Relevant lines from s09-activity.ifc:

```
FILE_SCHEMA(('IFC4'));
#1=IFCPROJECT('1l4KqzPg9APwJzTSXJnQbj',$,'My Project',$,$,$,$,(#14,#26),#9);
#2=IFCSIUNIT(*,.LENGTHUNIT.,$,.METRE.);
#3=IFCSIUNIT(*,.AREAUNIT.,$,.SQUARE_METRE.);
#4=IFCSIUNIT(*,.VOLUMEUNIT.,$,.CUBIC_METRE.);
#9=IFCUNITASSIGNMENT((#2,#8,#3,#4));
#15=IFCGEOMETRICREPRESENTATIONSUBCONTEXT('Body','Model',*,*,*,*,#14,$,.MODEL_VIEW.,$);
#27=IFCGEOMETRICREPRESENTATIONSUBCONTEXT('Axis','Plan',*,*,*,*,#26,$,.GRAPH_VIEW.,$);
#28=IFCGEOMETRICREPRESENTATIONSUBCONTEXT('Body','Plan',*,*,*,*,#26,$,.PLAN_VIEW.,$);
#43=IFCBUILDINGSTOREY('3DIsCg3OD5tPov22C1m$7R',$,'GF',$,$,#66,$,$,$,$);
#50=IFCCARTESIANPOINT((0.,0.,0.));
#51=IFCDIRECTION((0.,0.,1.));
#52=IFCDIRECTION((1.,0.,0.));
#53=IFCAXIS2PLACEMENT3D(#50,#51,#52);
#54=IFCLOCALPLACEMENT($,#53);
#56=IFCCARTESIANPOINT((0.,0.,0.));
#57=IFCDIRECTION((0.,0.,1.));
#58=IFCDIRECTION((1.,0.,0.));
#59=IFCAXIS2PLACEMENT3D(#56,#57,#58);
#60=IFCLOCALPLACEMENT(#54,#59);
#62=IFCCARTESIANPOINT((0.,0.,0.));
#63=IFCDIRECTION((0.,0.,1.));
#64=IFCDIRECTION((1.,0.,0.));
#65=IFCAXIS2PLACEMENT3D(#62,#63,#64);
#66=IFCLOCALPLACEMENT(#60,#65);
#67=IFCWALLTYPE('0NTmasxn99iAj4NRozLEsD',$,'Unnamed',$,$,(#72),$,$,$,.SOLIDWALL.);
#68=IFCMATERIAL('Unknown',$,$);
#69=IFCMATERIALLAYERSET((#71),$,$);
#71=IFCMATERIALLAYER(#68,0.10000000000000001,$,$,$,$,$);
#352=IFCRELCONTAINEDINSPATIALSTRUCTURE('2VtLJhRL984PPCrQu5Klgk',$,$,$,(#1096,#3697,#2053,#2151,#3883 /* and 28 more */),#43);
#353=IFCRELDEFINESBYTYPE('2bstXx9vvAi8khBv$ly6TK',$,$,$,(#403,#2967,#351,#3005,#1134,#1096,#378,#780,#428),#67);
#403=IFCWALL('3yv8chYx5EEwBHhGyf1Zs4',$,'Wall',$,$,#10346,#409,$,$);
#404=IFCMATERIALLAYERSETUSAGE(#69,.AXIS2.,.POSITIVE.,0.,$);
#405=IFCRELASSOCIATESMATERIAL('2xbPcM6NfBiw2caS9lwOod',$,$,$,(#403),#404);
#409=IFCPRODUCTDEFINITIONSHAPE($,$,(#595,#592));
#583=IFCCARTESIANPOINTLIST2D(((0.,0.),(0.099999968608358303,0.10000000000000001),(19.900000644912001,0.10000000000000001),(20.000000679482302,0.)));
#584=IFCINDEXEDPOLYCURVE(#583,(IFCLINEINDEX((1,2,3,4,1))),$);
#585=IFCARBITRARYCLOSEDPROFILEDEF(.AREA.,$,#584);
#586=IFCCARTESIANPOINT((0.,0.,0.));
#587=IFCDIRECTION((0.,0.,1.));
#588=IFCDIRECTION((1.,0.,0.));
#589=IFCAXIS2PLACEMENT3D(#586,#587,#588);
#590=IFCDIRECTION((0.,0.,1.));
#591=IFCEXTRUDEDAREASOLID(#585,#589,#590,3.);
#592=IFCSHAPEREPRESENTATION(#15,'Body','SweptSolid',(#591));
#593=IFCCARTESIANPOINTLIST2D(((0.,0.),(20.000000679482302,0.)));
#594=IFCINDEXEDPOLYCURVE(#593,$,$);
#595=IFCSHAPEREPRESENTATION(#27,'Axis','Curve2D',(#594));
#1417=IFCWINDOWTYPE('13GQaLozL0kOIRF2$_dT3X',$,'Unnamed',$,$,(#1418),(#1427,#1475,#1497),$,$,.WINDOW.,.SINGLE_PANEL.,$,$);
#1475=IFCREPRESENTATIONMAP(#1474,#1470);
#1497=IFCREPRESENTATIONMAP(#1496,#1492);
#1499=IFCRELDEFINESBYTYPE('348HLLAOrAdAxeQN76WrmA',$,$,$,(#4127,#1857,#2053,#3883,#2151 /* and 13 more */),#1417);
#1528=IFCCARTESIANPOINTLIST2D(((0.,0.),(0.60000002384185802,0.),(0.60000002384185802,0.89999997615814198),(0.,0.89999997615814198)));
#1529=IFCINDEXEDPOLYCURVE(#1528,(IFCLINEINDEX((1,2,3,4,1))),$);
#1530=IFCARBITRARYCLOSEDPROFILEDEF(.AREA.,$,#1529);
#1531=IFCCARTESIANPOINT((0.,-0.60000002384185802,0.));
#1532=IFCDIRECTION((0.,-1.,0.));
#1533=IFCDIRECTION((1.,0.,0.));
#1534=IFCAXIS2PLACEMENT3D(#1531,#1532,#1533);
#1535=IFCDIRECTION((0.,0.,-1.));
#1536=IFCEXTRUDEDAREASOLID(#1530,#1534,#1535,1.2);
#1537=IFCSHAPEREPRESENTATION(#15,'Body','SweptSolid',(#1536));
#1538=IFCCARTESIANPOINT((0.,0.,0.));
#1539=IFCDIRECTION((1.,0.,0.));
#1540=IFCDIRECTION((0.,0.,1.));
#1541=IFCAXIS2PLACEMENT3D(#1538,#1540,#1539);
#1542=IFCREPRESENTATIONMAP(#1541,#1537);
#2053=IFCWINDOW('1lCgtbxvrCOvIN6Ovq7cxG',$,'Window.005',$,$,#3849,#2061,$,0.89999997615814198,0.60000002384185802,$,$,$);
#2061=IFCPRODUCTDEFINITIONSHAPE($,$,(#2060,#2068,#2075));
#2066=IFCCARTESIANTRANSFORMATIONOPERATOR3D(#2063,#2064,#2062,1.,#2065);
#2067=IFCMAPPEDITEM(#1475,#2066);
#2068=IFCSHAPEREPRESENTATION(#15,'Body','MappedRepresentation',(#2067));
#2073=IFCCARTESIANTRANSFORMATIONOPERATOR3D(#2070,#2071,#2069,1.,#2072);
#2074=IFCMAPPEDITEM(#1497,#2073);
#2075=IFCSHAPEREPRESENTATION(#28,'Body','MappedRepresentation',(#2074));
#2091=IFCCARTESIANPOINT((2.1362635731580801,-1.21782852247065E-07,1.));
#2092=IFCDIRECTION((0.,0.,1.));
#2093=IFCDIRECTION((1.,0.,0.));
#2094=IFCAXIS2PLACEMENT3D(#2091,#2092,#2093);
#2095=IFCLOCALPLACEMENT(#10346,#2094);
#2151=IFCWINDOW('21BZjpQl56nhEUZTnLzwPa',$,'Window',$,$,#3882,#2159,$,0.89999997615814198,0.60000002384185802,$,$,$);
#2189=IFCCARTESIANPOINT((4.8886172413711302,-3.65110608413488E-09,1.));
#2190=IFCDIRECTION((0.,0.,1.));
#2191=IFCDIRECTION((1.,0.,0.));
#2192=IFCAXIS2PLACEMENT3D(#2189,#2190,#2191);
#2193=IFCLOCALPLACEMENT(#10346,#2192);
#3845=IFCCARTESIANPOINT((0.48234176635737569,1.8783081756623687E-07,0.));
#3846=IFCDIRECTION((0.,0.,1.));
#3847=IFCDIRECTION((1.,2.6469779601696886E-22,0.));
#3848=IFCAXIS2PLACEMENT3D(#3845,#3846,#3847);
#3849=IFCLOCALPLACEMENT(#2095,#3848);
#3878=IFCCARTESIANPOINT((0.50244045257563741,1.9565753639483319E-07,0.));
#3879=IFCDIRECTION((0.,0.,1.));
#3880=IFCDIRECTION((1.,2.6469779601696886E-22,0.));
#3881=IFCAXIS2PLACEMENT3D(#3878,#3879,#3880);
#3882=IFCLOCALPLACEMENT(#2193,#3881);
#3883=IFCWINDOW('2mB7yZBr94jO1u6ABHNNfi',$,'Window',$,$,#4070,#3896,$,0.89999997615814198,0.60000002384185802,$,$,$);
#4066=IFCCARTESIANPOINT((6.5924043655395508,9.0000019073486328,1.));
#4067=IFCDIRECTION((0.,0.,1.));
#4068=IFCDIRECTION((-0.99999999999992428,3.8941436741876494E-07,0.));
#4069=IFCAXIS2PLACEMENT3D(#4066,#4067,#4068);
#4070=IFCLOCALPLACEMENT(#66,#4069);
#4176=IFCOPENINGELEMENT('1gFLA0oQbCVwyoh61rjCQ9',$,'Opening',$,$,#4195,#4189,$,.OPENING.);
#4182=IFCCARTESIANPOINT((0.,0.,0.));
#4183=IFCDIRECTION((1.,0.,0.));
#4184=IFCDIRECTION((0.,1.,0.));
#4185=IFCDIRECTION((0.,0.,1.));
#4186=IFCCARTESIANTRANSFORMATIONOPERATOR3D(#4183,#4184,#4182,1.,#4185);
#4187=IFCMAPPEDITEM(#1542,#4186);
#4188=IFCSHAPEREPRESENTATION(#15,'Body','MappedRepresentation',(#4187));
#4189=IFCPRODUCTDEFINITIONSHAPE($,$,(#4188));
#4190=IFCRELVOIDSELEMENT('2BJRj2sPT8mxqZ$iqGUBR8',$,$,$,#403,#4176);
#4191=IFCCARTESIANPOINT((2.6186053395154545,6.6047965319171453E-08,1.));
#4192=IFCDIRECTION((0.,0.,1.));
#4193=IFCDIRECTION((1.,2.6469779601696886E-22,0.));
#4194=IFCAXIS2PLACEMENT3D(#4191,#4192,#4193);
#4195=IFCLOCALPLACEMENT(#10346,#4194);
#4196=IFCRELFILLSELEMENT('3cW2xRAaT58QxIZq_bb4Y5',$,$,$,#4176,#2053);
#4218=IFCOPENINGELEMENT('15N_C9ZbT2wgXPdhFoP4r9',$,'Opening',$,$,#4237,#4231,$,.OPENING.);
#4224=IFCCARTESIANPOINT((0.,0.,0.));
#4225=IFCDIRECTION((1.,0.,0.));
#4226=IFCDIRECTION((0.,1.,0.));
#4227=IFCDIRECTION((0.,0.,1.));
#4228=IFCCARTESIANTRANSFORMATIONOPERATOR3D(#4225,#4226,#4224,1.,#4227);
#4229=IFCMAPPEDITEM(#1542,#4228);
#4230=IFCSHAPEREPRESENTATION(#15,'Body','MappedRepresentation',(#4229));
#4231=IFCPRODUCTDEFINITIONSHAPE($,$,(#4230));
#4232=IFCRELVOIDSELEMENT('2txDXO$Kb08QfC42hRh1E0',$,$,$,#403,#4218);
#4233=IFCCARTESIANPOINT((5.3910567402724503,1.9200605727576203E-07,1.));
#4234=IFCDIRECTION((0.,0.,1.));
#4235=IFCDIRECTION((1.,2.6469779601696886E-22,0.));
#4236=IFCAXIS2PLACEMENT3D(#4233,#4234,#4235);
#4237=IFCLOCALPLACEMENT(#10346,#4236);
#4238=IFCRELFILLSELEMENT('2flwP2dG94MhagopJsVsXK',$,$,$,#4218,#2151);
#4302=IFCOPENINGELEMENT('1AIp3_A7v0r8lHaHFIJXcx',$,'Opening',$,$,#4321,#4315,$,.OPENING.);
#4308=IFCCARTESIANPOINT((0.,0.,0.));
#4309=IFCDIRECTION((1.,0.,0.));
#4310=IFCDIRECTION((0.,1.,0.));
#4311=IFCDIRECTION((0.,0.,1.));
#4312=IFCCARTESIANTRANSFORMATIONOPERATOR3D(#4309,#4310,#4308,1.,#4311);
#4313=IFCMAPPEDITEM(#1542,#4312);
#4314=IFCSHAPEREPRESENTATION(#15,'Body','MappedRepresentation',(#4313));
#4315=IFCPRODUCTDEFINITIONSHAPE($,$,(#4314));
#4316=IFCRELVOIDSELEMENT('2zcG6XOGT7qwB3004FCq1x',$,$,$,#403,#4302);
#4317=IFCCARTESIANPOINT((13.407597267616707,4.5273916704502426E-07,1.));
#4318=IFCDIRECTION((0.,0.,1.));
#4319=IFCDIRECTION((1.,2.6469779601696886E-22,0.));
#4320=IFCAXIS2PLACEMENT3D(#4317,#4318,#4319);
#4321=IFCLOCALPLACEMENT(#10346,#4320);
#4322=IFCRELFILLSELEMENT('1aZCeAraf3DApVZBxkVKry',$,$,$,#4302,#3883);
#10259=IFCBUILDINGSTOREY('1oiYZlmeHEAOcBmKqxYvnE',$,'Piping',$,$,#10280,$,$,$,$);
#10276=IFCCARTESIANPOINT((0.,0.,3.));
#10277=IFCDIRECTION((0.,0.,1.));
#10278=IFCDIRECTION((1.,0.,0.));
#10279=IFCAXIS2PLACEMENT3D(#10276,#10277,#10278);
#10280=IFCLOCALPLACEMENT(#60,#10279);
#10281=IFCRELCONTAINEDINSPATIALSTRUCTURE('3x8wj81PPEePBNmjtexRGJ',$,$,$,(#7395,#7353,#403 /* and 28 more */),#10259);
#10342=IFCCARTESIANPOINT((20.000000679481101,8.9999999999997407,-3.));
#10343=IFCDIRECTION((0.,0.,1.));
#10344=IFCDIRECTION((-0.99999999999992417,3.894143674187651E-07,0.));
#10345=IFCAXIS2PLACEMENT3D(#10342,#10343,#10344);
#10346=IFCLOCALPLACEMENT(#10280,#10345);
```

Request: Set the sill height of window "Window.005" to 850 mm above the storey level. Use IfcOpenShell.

```python
import numpy as np
import ifcopenshell
import ifcopenshell.api.geometry
import ifcopenshell.geom
import ifcopenshell.util.element
import ifcopenshell.util.placement
import ifcopenshell.util.shape
import ifcopenshell.util.unit

model = ifcopenshell.open("s09-activity.ifc")
unit_scale = ifcopenshell.util.unit.calculate_unit_scale(model)

window = model.by_guid("1lCgtbxvrCOvIN6Ovq7cxG")
opening = window.FillsVoids[0].RelatingOpeningElement
storey = ifcopenshell.util.element.get_container(window, ifc_class="IfcBuildingStorey")
level = ifcopenshell.util.placement.get_local_placement(storey.ObjectPlacement)[2, 3]

# The opening's origin need not be at the sill, so measure its lowest point.
shape = ifcopenshell.geom.create_shape(ifcopenshell.geom.settings(), opening)
bottom = ifcopenshell.util.shape.get_shape_bottom_elevation(shape, shape.geometry) / unit_scale
dz = level + 0.85 / unit_scale - bottom

shift = np.array([0.0, 0.0, dz])
# The window is not placed relative to its opening, so move both.
for product in (opening, window):
    matrix = ifcopenshell.util.placement.get_local_placement(product.ObjectPlacement)
    matrix[:3, 3] += shift
    ifcopenshell.api.geometry.edit_object_placement(model, product=product, matrix=matrix, is_si=False)

print(f"moved by {dz * unit_scale:+.3f} m")

model.write("s09-activity_rev.ifc")
```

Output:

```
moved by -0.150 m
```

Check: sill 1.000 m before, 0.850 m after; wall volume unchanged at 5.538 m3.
